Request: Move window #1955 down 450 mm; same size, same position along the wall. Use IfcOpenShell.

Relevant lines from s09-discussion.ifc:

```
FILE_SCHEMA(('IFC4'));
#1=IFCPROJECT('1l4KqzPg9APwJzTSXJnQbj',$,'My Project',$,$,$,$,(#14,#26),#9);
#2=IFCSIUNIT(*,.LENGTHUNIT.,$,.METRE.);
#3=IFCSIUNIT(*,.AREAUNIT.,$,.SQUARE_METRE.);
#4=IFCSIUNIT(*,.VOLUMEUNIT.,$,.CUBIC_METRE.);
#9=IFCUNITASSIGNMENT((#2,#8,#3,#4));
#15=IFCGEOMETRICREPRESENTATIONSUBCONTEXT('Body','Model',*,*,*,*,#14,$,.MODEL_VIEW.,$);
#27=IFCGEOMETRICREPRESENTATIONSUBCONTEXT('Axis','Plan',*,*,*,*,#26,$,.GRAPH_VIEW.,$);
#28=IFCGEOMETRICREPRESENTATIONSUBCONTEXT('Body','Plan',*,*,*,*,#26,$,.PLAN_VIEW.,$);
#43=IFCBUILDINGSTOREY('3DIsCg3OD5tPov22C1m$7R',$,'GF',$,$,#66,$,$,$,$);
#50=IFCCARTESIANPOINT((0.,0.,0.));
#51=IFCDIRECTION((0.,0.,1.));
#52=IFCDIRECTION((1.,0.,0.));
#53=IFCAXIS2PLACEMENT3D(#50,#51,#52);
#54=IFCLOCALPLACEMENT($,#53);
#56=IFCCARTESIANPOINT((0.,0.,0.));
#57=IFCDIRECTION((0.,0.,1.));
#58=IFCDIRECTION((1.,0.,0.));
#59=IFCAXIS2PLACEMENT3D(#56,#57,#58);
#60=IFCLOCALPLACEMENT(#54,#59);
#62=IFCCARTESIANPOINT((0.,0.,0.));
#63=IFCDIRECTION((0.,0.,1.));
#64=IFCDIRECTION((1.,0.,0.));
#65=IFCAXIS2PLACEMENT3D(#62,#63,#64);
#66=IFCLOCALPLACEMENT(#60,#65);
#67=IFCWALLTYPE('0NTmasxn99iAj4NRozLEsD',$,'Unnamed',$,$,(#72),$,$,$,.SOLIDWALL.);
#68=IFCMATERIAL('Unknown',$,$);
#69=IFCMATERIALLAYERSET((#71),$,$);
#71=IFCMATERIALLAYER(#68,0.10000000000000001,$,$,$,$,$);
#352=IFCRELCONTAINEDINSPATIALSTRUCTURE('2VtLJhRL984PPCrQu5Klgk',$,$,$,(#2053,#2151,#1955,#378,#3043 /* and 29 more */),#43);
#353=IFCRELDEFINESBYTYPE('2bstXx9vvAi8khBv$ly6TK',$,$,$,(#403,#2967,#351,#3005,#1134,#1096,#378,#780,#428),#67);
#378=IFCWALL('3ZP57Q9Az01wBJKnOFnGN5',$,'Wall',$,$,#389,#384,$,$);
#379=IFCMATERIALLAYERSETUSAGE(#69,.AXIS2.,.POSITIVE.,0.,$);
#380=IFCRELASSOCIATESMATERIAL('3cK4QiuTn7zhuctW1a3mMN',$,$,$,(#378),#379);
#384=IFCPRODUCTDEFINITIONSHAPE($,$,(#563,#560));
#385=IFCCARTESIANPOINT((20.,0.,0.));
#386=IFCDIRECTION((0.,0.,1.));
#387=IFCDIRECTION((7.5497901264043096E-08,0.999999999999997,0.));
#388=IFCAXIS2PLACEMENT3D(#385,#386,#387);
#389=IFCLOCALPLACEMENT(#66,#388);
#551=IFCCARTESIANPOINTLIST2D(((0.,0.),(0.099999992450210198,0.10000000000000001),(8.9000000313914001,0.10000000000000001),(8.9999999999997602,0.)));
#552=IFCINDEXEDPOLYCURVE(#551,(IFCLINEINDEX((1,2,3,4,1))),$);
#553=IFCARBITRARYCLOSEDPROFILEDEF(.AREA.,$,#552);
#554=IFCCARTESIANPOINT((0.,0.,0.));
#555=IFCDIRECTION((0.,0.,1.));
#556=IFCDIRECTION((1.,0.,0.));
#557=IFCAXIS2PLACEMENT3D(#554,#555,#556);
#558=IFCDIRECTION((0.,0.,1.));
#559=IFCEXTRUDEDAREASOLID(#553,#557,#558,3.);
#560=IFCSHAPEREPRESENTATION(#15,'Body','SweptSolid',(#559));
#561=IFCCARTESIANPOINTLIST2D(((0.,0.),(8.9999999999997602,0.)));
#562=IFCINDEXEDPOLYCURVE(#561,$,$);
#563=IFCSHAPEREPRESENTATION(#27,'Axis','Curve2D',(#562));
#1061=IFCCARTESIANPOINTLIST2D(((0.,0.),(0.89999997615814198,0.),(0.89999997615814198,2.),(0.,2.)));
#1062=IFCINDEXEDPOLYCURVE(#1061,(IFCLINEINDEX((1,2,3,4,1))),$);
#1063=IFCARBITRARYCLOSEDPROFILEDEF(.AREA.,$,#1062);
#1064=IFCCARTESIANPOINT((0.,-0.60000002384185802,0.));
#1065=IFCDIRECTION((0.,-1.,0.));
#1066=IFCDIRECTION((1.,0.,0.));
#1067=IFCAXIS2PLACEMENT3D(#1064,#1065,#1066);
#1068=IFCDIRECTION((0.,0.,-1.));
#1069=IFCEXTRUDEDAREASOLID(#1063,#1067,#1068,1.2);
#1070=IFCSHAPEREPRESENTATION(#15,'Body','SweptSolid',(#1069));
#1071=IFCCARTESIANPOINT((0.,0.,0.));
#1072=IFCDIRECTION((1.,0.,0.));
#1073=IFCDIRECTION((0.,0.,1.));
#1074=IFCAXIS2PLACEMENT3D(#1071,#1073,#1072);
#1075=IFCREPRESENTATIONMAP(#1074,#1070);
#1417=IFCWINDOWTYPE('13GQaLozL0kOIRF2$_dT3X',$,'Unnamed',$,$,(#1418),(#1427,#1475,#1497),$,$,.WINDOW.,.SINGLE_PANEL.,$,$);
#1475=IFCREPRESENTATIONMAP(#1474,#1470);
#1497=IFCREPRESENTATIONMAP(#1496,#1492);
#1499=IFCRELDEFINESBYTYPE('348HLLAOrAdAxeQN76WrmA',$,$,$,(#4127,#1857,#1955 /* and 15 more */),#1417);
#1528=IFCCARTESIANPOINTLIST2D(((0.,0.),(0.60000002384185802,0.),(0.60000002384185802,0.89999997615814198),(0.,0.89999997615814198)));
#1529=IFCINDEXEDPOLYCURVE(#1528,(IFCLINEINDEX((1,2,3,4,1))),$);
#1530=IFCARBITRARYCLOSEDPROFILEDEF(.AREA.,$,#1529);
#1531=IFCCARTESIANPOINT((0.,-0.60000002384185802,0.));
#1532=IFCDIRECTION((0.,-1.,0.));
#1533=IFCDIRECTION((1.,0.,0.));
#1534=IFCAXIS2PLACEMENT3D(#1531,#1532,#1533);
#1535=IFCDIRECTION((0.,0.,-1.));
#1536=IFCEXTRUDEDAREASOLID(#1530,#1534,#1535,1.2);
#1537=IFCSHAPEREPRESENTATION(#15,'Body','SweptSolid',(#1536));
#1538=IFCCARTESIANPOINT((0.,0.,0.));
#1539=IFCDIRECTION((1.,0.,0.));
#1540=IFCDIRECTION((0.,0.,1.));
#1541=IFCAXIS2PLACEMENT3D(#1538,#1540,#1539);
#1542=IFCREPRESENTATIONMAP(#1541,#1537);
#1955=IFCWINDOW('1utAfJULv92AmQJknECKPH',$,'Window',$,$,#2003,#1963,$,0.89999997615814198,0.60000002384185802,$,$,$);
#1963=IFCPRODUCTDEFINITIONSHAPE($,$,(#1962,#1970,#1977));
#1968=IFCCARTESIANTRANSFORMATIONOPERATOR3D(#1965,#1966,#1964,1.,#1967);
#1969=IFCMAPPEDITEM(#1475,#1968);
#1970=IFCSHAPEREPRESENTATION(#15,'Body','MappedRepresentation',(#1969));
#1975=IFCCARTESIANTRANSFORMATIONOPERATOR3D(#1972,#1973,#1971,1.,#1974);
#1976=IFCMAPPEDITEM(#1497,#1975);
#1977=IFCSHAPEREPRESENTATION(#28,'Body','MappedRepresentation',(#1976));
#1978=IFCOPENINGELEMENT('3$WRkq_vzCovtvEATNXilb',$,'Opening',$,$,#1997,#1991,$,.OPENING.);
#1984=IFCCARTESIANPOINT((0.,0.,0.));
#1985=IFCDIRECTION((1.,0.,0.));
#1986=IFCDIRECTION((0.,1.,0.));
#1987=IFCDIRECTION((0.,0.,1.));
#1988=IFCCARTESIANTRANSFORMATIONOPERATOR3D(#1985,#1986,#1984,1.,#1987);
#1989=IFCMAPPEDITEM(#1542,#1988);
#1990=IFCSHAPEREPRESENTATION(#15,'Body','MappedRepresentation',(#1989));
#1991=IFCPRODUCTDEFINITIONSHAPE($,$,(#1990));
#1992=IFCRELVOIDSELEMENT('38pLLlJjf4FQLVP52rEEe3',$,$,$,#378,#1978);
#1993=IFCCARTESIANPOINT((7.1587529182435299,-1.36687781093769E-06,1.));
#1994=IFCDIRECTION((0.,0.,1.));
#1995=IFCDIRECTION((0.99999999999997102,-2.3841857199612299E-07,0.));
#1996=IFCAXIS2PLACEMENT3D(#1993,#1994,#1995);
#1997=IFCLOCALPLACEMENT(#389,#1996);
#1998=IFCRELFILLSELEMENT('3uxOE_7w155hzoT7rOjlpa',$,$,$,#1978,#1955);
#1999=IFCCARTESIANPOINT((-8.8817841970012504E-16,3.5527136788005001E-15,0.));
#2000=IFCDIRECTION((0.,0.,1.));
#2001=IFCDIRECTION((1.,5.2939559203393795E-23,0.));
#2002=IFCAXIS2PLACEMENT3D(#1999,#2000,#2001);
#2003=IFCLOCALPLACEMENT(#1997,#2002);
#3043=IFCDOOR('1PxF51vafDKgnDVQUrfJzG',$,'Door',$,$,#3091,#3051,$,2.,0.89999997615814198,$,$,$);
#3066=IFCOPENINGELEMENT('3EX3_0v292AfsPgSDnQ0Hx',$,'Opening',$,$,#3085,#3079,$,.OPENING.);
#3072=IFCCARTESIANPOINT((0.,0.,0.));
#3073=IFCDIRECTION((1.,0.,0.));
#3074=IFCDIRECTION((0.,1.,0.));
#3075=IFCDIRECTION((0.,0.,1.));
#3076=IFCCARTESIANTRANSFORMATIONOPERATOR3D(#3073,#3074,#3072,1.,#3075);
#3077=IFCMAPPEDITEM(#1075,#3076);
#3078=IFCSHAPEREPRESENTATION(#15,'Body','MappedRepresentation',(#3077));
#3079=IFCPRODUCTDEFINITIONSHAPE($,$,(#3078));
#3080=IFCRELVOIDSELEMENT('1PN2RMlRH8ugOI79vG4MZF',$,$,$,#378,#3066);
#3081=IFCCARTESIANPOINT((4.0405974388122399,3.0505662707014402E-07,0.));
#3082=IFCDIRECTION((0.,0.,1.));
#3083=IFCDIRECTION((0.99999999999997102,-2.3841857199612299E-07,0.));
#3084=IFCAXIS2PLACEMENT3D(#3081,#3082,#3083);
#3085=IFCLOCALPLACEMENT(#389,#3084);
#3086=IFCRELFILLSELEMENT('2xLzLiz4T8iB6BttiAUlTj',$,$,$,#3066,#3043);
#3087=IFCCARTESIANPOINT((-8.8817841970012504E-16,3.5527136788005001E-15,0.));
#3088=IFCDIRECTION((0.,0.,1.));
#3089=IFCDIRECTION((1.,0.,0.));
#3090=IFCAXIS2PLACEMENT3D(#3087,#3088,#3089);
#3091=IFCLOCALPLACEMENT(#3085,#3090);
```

```python
import numpy as np
import ifcopenshell
import ifcopenshell.api.geometry
import ifcopenshell.util.placement
import ifcopenshell.util.unit

model = ifcopenshell.open("s09-discussion.ifc")
unit_scale = ifcopenshell.util.unit.calculate_unit_scale(model)

window = model.by_guid("1utAfJULv92AmQJknECKPH")
opening = window.FillsVoids[0].RelatingOpeningElement
dz = -0.45 / unit_scale

shift = np.array([0.0, 0.0, dz])
# The window is placed relative to its opening, so it follows when the opening moves.
matrix = ifcopenshell.util.placement.get_local_placement(opening.ObjectPlacement)
matrix[:3, 3] += shift
ifcopenshell.api.geometry.edit_object_placement(
    model, product=opening, matrix=matrix, is_si=False, should_transform_children=True
)

print(f"moved by {dz * unit_scale:+.3f} m")

model.write("s09-discussion_edited.ifc")
```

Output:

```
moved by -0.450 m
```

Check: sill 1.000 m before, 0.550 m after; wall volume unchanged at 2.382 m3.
